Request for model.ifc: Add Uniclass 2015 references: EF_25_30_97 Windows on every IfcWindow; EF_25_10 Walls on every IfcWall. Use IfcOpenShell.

First a look at what the model holds.

```python
import ifcopenshell

model = ifcopenshell.open("model.ifc")
print(model.schema)
print("classifications:", [c.Name for c in model.by_type("IfcClassification")])
for ifc_class in ("IfcDoor", "IfcRoof", "IfcStair", "IfcWall", "IfcWindow"):
    print(ifc_class, len(model.by_type(ifc_class)))
```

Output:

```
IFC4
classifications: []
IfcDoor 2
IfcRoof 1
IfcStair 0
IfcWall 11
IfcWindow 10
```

```python
import ifcopenshell
import ifcopenshell.api.classification

model = ifcopenshell.open("model.ifc")

system = ifcopenshell.api.classification.add_classification(model, classification="Uniclass 2015")

codes = {
    "IfcWindow": ("EF_25_30_97", "Windows"),
    "IfcWall": ("EF_25_10", "Walls"),
}
for ifc_class, (code, name) in codes.items():
    products = model.by_type(ifc_class)
    ifcopenshell.api.classification.add_reference(
        model, products=products, classification=system, identification=code, name=name
    )
    print(code, len(products))

model.write("model_v2.ifc")
```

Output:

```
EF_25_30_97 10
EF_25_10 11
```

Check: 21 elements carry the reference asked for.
